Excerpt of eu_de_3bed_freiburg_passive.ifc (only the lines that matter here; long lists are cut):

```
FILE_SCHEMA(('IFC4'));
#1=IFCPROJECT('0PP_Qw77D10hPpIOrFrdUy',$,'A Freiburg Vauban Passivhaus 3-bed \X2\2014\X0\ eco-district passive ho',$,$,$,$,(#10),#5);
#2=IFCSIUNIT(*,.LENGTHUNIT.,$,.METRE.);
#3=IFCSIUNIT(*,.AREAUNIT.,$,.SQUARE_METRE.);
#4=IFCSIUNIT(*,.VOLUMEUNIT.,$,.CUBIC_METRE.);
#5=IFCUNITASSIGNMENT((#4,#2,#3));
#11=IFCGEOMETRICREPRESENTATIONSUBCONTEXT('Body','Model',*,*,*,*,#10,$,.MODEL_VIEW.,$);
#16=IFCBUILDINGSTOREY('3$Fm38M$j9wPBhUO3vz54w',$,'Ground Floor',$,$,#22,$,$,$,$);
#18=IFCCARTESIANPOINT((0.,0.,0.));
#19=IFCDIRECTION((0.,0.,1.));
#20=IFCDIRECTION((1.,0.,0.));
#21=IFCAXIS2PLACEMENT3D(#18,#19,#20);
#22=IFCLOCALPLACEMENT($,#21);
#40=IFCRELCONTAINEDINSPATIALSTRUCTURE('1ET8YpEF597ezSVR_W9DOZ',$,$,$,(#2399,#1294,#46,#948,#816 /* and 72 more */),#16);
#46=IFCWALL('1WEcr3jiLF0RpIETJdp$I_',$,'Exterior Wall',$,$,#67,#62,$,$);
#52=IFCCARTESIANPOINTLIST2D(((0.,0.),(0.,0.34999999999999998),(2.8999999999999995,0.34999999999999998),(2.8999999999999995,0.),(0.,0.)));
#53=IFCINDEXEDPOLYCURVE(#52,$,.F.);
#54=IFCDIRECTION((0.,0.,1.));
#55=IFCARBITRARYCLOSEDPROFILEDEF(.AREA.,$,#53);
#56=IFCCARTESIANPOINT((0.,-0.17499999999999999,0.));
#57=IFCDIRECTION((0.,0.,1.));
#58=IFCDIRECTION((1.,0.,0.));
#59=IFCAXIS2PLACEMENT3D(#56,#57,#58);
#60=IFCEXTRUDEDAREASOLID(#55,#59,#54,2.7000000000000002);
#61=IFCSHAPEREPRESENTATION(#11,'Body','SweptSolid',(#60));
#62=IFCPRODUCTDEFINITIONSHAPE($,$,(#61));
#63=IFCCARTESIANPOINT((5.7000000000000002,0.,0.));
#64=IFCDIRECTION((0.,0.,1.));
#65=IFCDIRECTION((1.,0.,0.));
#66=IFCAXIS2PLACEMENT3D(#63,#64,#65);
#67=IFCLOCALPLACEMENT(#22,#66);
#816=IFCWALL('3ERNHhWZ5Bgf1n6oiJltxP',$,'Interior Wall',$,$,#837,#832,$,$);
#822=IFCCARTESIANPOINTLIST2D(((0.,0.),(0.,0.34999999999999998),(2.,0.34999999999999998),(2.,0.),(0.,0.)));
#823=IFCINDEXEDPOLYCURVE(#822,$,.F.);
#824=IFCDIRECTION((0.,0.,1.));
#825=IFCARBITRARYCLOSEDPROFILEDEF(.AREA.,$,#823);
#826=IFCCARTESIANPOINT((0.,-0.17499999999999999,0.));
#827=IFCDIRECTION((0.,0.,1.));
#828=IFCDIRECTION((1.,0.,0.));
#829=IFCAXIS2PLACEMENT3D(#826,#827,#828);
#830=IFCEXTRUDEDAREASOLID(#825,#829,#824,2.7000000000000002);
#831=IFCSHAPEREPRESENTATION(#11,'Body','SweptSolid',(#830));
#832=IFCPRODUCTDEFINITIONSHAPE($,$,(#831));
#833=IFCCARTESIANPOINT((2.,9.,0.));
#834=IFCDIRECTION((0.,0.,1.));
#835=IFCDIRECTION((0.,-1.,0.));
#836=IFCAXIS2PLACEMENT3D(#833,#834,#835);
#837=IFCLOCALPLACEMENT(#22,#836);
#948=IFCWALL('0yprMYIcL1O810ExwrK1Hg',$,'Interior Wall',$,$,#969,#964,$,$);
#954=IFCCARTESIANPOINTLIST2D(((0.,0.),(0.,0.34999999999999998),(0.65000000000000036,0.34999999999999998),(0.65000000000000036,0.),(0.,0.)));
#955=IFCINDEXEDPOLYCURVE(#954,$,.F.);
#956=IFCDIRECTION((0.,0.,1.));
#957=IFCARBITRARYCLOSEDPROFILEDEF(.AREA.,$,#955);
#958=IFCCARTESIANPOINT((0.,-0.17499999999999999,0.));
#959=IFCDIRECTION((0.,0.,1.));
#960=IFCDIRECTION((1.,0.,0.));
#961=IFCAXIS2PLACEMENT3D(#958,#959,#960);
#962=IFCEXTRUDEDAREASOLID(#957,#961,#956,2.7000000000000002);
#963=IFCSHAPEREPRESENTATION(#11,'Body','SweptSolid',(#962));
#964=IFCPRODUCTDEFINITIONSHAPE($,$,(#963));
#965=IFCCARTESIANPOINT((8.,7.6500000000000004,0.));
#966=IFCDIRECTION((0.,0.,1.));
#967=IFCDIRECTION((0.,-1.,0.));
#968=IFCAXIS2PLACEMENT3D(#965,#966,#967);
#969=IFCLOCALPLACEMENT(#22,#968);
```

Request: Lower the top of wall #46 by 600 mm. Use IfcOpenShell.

```python
import ifcopenshell
import ifcopenshell.geom
import ifcopenshell.util.representation
import ifcopenshell.util.shape

model = ifcopenshell.open("eu_de_3bed_freiburg_passive.ifc")
settings = ifcopenshell.geom.settings()


def volume(element):
    """Net volume in cubic metres, openings subtracted."""
    shape = ifcopenshell.geom.create_shape(settings, element)
    return ifcopenshell.util.shape.get_volume(shape.geometry)


wall = model.by_guid("1WEcr3jiLF0RpIETJdp$I_")
before = volume(wall)

body = ifcopenshell.util.representation.get_representation(wall, "Model", "Body")
solid = body.Items[0]
old_height = solid.Depth
solid.Depth -= 0.6
after = volume(wall)

print(f"height {old_height:g} -> {solid.Depth:g}, volume {before:.3f} -> {after:.3f} m3")

model.write("eu_de_3bed_freiburg_passive-out.ifc")
```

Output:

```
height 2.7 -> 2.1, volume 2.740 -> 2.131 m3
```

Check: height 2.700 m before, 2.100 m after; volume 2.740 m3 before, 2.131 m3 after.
